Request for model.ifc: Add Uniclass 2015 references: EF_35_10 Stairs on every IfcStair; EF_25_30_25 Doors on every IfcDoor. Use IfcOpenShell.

First a look at what the model holds.

```python
import ifcopenshell

model = ifcopenshell.open("model.ifc")
print(model.schema)
print("classifications:", [c.Name for c in model.by_type("IfcClassification")])
for ifc_class in ("IfcDoor", "IfcRoof", "IfcStair", "IfcWall", "IfcWindow"):
    print(ifc_class, len(model.by_type(ifc_class)))
```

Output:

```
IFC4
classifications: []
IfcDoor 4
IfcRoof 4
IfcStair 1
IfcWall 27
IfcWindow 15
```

```python
import ifcopenshell
import ifcopenshell.api.classification

model = ifcopenshell.open("model.ifc")

system = ifcopenshell.api.classification.add_classification(model, classification="Uniclass 2015")

codes = {
    "IfcStair": ("EF_35_10", "Stairs"),
    "IfcDoor": ("EF_25_30_25", "Doors"),
}
for ifc_class, (code, name) in codes.items():
    products = model.by_type(ifc_class)
    ifcopenshell.api.classification.add_reference(
        model, products=products, classification=system, identification=code, name=name
    )
    print(code, len(products))

model.write("model_v2.ifc")
```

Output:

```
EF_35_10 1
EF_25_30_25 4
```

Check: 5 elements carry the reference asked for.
